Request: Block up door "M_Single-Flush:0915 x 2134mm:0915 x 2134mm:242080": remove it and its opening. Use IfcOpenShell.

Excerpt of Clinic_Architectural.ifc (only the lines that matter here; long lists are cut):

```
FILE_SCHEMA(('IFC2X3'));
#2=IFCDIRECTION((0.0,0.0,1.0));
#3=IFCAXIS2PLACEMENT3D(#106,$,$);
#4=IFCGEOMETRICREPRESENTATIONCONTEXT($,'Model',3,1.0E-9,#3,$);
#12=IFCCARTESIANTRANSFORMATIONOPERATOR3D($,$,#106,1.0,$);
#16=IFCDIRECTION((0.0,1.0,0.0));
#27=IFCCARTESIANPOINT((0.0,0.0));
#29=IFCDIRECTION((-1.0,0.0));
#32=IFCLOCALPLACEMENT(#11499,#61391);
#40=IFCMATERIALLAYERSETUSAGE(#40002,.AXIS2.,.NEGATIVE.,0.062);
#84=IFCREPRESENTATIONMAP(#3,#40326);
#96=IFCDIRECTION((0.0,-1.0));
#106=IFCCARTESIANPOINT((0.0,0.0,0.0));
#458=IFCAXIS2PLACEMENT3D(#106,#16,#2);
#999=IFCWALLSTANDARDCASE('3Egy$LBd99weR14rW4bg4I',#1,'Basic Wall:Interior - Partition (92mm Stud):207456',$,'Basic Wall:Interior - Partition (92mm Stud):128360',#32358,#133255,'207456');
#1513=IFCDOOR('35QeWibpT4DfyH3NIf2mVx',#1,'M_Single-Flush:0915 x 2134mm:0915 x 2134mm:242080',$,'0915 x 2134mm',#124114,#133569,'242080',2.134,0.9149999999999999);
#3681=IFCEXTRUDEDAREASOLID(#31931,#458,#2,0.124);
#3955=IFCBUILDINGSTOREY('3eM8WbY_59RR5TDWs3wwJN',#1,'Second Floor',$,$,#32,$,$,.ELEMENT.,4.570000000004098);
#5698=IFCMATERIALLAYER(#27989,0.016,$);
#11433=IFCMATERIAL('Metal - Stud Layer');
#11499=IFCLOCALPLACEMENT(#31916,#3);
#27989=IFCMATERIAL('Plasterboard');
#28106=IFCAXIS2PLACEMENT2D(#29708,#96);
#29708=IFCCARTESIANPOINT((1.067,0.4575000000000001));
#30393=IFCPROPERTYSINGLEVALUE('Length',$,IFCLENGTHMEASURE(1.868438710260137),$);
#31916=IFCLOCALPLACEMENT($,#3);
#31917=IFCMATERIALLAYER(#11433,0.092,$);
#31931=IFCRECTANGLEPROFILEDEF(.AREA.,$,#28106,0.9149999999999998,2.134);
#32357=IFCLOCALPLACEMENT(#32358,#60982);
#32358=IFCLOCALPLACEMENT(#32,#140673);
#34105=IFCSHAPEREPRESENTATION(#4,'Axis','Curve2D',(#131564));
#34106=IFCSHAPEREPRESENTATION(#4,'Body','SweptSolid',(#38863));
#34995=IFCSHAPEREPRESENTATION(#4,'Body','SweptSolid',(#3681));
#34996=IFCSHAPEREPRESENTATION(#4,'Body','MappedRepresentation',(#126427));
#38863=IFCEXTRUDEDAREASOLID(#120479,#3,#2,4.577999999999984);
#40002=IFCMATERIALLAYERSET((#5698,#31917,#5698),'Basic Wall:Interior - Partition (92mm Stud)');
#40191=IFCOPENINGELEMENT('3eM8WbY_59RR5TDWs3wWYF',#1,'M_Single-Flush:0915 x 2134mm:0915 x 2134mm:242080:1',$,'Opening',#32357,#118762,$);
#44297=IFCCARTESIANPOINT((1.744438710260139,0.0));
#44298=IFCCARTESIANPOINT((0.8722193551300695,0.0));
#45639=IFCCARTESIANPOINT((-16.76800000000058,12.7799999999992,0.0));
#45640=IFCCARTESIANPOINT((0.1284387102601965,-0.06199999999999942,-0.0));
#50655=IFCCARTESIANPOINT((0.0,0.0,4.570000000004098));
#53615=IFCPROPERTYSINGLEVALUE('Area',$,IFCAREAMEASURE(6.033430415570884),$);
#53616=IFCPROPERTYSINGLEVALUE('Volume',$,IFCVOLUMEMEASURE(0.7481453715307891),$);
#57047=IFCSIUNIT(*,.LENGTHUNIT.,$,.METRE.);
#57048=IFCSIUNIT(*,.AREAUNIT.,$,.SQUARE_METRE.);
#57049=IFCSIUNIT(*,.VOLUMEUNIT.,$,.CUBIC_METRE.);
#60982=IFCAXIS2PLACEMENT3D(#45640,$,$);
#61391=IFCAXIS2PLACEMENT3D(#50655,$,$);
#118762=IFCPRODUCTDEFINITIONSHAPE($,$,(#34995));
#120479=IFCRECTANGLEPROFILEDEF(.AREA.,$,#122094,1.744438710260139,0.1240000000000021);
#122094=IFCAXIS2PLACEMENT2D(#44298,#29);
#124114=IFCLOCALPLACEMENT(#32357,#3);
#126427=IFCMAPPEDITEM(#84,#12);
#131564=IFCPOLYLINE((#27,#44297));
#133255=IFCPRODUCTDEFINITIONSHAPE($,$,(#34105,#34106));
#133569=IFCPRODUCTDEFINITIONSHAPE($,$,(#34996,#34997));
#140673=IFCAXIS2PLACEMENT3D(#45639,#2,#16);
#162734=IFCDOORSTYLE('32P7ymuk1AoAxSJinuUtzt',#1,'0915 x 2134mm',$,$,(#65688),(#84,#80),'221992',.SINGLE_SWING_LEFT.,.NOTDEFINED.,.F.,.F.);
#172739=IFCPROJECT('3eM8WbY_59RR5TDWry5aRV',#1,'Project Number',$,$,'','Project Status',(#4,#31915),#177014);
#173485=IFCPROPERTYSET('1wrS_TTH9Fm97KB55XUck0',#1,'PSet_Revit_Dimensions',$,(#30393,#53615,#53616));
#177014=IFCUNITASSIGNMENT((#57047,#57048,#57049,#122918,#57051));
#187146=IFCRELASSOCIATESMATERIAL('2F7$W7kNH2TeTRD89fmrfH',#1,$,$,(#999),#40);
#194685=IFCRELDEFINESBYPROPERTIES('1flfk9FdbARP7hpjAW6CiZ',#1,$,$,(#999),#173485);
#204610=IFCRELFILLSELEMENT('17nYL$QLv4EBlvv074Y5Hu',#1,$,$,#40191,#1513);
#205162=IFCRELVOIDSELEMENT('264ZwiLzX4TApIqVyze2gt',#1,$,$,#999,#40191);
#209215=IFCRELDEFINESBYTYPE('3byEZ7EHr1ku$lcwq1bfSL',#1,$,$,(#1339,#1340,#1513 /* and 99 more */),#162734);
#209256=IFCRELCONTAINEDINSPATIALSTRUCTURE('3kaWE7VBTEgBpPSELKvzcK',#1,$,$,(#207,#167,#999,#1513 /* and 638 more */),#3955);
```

```python
import ifcopenshell
import ifcopenshell.api.feature
import ifcopenshell.api.pset
import ifcopenshell.api.root
import ifcopenshell.geom
import ifcopenshell.util.element
import ifcopenshell.util.shape
import ifcopenshell.util.unit

model = ifcopenshell.open("Clinic_Architectural.ifc")
area_scale = ifcopenshell.util.unit.calculate_unit_scale(model, "AREAUNIT")
volume_scale = ifcopenshell.util.unit.calculate_unit_scale(model, "VOLUMEUNIT")
settings = ifcopenshell.geom.settings()


def volume(element):
    """Net volume in cubic metres, openings subtracted."""
    shape = ifcopenshell.geom.create_shape(settings, element)
    return ifcopenshell.util.shape.get_volume(shape.geometry)


door = model.by_guid("35QeWibpT4DfyH3NIf2mVx")
opening = door.FillsVoids[0].RelatingOpeningElement
wall = opening.VoidsElements[0].RelatingBuildingElement
before = volume(wall)

ifcopenshell.api.root.remove_product(model, product=door)
ifcopenshell.api.feature.remove_feature(model, feature=opening)

after = volume(wall)
thickness = 0.124  # wall thickness in metres

# Update the wall's stored quantities.
pset = model.by_id(ifcopenshell.util.element.get_pset(wall, "PSet_Revit_Dimensions", should_inherit=False)["id"])
ifcopenshell.api.pset.edit_pset(model, pset=pset, properties={
    "Area": model.create_entity("IfcAreaMeasure", after / thickness / area_scale),
    "Volume": model.create_entity("IfcVolumeMeasure", after / volume_scale),
})

print(f"wall volume {before:.3f} -> {after:.3f} m3")

model.write("Clinic_Architectural_v2.ifc")
```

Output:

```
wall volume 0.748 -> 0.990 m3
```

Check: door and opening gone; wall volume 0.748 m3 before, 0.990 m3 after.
